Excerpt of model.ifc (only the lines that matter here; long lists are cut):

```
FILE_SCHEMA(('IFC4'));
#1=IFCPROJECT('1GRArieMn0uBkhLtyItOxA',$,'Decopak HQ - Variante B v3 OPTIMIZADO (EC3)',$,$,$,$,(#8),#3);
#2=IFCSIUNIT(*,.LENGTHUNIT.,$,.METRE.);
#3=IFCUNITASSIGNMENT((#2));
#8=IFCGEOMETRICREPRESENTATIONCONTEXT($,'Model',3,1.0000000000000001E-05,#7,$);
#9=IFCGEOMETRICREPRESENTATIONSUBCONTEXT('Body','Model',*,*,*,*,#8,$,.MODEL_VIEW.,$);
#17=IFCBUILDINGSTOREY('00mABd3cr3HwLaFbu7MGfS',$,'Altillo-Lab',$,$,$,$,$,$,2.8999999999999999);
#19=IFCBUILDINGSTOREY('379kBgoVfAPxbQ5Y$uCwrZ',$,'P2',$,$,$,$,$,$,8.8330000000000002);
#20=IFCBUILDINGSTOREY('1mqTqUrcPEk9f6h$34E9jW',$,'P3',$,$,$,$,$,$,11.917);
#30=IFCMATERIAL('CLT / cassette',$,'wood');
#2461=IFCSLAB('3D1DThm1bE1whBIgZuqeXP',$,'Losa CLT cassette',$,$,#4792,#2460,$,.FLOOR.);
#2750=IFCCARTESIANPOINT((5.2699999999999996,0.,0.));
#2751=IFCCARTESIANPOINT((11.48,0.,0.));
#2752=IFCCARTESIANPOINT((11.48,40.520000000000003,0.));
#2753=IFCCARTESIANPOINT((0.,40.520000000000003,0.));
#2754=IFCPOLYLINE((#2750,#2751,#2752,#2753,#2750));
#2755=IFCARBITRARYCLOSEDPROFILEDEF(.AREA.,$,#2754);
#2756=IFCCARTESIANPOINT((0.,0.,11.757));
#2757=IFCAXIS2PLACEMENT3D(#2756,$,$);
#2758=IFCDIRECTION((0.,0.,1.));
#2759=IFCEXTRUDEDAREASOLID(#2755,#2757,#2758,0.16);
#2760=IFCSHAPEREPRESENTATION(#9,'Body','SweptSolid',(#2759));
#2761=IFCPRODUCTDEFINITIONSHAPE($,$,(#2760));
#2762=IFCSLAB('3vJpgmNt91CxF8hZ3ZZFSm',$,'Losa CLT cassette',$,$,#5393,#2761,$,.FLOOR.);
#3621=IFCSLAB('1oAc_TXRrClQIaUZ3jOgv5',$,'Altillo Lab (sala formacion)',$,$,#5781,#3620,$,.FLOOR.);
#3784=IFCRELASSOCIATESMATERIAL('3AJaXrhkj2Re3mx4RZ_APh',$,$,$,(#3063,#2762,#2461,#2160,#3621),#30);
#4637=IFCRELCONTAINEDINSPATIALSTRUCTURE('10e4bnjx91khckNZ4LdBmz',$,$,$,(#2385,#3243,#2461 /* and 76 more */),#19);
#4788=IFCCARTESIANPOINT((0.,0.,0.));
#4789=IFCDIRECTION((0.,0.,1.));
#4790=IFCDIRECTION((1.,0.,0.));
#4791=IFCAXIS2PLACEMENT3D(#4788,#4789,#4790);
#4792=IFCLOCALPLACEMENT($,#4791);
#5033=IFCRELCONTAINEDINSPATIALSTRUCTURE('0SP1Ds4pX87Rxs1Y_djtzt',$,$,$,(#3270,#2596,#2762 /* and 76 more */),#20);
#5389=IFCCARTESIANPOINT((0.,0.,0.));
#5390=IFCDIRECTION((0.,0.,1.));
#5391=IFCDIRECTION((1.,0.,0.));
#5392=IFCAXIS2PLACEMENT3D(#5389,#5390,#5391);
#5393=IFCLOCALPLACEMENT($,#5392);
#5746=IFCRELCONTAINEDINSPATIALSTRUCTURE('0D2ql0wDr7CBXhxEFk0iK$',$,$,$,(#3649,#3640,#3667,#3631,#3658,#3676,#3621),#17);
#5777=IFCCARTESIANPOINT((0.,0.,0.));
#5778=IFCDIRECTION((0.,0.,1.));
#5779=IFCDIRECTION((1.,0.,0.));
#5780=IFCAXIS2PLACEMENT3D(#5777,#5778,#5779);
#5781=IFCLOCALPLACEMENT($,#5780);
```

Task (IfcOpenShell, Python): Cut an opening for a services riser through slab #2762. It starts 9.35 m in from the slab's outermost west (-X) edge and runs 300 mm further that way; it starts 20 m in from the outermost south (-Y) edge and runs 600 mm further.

```python
import numpy as np
import ifcopenshell
import ifcopenshell.api.feature
import ifcopenshell.api.geometry
import ifcopenshell.api.root
import ifcopenshell.geom
import ifcopenshell.util.placement
import ifcopenshell.util.representation
import ifcopenshell.util.shape
import ifcopenshell.util.unit

model = ifcopenshell.open("model.ifc")
unit_scale = ifcopenshell.util.unit.calculate_unit_scale(model)
settings = ifcopenshell.geom.settings()


def volume(element):
    """Net volume in cubic metres, openings subtracted."""
    shape = ifcopenshell.geom.create_shape(settings, element)
    return ifcopenshell.util.shape.get_volume(shape.geometry)


slab = model.by_guid("3vJpgmNt91CxF8hZ3ZZFSm")
before = volume(slab)

# Extent in the slab's own axes, in metres. The edges named are its -X and -Y sides.
slab_shape = ifcopenshell.geom.create_shape(settings, slab)
vertices = ifcopenshell.util.shape.get_vertices(slab_shape.geometry)
x_min, y_min, bottom = vertices.min(axis=0)
top = vertices[:, 2].max()

opening = ifcopenshell.api.root.create_entity(model, ifc_class="IfcOpeningElement", name="Services riser opening", predefined_type="OPENING")
context = ifcopenshell.util.representation.get_context(model, "Model", "Body", "MODEL_VIEW")
width, depth = 0.3, 0.6
outline = [(0.0, 0.0), (width, 0.0), (width, depth), (0.0, depth), (0.0, 0.0)]
# Overshoot both faces by 50 mm so the cut is clean.
shape = ifcopenshell.api.geometry.add_slab_representation(
    model, context=context, depth=top - bottom + 0.1, polyline=outline
)
ifcopenshell.api.geometry.assign_representation(model, product=opening, representation=shape)

matrix = ifcopenshell.util.placement.get_local_placement(slab.ObjectPlacement)
matrix[:, 3] = matrix @ np.append(np.array([x_min + 9.35, y_min + 20, bottom - 0.05]) / unit_scale, 1.0)
ifcopenshell.api.geometry.edit_object_placement(model, product=opening, matrix=matrix, is_si=False)
ifcopenshell.api.feature.add_feature(model, feature=opening, element=slab)

after = volume(slab)

print(f"slab volume {before:.3f} -> {after:.3f} m3")

model.write("model_edited.ifc")
```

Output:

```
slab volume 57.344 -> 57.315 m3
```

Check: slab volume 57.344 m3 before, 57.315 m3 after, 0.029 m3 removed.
